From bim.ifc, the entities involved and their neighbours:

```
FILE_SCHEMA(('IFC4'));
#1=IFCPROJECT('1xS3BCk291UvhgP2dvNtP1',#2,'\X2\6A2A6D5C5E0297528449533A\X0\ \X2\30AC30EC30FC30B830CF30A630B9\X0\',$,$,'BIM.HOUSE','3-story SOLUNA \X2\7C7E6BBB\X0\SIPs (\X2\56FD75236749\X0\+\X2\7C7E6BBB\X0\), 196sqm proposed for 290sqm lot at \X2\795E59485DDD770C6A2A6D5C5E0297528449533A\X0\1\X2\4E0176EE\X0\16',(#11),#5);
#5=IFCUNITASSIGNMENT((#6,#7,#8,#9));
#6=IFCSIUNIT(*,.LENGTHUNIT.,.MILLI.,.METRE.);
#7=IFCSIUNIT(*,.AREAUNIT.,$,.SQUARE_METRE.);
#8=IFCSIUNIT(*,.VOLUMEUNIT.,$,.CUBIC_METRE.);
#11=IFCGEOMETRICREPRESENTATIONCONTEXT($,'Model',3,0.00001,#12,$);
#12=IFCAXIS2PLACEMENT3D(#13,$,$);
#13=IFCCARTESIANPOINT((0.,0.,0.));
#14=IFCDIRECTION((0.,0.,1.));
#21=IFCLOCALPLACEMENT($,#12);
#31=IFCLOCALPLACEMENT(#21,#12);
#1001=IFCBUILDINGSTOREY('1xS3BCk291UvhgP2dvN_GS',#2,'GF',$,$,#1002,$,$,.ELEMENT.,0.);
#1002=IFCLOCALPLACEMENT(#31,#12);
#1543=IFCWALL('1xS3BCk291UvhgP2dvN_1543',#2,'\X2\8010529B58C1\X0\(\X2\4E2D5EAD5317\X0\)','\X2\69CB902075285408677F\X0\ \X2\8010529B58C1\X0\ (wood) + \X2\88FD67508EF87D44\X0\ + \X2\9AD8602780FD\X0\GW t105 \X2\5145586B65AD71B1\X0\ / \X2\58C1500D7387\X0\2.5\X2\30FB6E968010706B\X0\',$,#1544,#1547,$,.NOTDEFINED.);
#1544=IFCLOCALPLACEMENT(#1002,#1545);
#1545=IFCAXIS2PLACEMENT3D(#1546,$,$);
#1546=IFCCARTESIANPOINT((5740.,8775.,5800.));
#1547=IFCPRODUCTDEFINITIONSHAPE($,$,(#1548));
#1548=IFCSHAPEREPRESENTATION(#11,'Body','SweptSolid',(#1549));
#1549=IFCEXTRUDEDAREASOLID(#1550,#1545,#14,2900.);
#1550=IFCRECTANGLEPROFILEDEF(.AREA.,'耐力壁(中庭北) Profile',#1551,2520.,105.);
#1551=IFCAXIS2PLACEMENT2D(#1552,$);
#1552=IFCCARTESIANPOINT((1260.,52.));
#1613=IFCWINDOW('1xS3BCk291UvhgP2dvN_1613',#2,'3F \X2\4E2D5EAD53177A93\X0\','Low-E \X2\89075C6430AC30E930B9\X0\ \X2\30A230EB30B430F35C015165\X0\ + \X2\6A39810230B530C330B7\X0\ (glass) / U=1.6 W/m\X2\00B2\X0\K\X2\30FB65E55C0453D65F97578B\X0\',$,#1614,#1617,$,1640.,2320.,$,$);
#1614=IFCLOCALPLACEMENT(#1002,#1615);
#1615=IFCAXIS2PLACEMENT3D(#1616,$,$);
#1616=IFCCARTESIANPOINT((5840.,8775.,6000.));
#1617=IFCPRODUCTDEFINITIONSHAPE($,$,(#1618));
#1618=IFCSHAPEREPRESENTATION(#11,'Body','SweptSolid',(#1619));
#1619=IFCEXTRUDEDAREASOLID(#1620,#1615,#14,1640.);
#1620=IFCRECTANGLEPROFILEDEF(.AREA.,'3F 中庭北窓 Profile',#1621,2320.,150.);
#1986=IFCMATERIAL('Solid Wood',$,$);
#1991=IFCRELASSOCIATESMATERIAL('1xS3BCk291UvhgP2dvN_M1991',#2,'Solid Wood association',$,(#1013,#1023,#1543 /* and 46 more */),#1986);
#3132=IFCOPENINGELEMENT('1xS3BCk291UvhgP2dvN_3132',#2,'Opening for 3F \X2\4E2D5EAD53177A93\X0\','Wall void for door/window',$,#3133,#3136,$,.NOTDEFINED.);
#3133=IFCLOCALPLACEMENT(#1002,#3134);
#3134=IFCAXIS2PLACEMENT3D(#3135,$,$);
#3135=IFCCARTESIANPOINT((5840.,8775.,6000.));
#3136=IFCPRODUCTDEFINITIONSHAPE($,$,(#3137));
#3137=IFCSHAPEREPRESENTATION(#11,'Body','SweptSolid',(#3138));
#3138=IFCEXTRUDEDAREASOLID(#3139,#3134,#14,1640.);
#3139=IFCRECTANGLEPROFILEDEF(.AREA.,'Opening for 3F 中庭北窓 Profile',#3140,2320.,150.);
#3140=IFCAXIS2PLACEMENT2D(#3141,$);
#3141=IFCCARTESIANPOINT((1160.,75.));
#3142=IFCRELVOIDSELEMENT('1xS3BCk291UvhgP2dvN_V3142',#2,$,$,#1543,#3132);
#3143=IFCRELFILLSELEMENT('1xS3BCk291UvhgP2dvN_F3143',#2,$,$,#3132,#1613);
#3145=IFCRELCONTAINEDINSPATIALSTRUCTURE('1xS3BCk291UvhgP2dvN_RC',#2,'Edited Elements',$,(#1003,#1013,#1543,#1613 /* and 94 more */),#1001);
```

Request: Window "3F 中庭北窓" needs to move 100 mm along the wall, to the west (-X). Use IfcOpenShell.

```python
import ifcopenshell
import ifcopenshell.api.geometry
import ifcopenshell.util.placement
import ifcopenshell.util.unit

model = ifcopenshell.open("bim.ifc")
unit_scale = ifcopenshell.util.unit.calculate_unit_scale(model)

window = model.by_guid("1xS3BCk291UvhgP2dvN_1613")
opening = window.FillsVoids[0].RelatingOpeningElement
wall = opening.VoidsElements[0].RelatingBuildingElement

wall_matrix = ifcopenshell.util.placement.get_local_placement(wall.ObjectPlacement)
shift = wall_matrix[:3, 0] * -0.1 / unit_scale
before = ifcopenshell.util.placement.get_local_placement(window.ObjectPlacement)[:3, 3].copy()

# The window is not placed relative to its opening, so move both.
for product in (opening, window):
    matrix = ifcopenshell.util.placement.get_local_placement(product.ObjectPlacement)
    matrix[:3, 3] += shift
    ifcopenshell.api.geometry.edit_object_placement(model, product=product, matrix=matrix, is_si=False)

after = ifcopenshell.util.placement.get_local_placement(window.ObjectPlacement)[:3, 3]
print("window moved by", (after - before).round(3) + 0.0)

model.write("bim-out.ifc")
```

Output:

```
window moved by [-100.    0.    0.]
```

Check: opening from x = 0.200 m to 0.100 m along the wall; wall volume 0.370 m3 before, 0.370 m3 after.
